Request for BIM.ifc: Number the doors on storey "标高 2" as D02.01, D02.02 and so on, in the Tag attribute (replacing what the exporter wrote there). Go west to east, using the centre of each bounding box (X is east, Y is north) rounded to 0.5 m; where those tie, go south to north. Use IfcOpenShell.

First a look at what the model holds.

```python
import ifcopenshell
import ifcopenshell.util.element
import ifcopenshell.util.placement

model = ifcopenshell.open("BIM.ifc")
print(model.schema)
storey = next(s for s in model.by_type("IfcBuildingStorey") if s.Name == "标高 2")
doors = [e for e in ifcopenshell.util.element.get_decomposition(storey) if e.is_a("IfcDoor")]
for e in sorted(doors, key=lambda e: e.id()):
    origin = ifcopenshell.util.placement.get_local_placement(e.ObjectPlacement)[:3, 3]
    print(e.id(), e.Tag, e.Name, origin.round(2) + 0.0, sep=" | ")
```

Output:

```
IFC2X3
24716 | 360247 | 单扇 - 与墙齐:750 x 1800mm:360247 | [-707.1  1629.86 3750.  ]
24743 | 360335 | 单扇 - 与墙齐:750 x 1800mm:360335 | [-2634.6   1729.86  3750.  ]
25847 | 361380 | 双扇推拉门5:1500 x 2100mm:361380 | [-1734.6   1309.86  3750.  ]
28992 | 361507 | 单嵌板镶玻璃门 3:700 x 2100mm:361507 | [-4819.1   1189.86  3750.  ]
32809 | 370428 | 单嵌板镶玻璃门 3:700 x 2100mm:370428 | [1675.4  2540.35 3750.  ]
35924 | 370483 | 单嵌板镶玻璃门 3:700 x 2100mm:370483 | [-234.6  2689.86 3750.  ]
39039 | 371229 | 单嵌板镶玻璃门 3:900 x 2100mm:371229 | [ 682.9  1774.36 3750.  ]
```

```python
import ifcopenshell
import ifcopenshell.geom
import ifcopenshell.util.element
import ifcopenshell.util.shape

model = ifcopenshell.open("BIM.ifc")
settings = ifcopenshell.geom.settings()
settings.set("use-world-coords", True)


def centre(element):
    shape = ifcopenshell.geom.create_shape(settings, element)
    return ifcopenshell.util.shape.get_bbox_centroid(shape.geometry)


storey = next(s for s in model.by_type("IfcBuildingStorey") if s.Name == "标高 2")
doors = [e for e in ifcopenshell.util.element.get_decomposition(storey) if e.is_a("IfcDoor")]

# Insertion points can sit at a corner or the storey origin, so sort by the geometry (in metres).
centres = {e: centre(e) for e in doors}
doors.sort(key=lambda e: (round(centres[e][0] / 0.5), centres[e][1]))

for i, e in enumerate(doors, start=1):
    number = f"D02.{i:02d}"
    e.Tag = number
    print(e.id(), number)

model.write("BIM_updated.ifc")
```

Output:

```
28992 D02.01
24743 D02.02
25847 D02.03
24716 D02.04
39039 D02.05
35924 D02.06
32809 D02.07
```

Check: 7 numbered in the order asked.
